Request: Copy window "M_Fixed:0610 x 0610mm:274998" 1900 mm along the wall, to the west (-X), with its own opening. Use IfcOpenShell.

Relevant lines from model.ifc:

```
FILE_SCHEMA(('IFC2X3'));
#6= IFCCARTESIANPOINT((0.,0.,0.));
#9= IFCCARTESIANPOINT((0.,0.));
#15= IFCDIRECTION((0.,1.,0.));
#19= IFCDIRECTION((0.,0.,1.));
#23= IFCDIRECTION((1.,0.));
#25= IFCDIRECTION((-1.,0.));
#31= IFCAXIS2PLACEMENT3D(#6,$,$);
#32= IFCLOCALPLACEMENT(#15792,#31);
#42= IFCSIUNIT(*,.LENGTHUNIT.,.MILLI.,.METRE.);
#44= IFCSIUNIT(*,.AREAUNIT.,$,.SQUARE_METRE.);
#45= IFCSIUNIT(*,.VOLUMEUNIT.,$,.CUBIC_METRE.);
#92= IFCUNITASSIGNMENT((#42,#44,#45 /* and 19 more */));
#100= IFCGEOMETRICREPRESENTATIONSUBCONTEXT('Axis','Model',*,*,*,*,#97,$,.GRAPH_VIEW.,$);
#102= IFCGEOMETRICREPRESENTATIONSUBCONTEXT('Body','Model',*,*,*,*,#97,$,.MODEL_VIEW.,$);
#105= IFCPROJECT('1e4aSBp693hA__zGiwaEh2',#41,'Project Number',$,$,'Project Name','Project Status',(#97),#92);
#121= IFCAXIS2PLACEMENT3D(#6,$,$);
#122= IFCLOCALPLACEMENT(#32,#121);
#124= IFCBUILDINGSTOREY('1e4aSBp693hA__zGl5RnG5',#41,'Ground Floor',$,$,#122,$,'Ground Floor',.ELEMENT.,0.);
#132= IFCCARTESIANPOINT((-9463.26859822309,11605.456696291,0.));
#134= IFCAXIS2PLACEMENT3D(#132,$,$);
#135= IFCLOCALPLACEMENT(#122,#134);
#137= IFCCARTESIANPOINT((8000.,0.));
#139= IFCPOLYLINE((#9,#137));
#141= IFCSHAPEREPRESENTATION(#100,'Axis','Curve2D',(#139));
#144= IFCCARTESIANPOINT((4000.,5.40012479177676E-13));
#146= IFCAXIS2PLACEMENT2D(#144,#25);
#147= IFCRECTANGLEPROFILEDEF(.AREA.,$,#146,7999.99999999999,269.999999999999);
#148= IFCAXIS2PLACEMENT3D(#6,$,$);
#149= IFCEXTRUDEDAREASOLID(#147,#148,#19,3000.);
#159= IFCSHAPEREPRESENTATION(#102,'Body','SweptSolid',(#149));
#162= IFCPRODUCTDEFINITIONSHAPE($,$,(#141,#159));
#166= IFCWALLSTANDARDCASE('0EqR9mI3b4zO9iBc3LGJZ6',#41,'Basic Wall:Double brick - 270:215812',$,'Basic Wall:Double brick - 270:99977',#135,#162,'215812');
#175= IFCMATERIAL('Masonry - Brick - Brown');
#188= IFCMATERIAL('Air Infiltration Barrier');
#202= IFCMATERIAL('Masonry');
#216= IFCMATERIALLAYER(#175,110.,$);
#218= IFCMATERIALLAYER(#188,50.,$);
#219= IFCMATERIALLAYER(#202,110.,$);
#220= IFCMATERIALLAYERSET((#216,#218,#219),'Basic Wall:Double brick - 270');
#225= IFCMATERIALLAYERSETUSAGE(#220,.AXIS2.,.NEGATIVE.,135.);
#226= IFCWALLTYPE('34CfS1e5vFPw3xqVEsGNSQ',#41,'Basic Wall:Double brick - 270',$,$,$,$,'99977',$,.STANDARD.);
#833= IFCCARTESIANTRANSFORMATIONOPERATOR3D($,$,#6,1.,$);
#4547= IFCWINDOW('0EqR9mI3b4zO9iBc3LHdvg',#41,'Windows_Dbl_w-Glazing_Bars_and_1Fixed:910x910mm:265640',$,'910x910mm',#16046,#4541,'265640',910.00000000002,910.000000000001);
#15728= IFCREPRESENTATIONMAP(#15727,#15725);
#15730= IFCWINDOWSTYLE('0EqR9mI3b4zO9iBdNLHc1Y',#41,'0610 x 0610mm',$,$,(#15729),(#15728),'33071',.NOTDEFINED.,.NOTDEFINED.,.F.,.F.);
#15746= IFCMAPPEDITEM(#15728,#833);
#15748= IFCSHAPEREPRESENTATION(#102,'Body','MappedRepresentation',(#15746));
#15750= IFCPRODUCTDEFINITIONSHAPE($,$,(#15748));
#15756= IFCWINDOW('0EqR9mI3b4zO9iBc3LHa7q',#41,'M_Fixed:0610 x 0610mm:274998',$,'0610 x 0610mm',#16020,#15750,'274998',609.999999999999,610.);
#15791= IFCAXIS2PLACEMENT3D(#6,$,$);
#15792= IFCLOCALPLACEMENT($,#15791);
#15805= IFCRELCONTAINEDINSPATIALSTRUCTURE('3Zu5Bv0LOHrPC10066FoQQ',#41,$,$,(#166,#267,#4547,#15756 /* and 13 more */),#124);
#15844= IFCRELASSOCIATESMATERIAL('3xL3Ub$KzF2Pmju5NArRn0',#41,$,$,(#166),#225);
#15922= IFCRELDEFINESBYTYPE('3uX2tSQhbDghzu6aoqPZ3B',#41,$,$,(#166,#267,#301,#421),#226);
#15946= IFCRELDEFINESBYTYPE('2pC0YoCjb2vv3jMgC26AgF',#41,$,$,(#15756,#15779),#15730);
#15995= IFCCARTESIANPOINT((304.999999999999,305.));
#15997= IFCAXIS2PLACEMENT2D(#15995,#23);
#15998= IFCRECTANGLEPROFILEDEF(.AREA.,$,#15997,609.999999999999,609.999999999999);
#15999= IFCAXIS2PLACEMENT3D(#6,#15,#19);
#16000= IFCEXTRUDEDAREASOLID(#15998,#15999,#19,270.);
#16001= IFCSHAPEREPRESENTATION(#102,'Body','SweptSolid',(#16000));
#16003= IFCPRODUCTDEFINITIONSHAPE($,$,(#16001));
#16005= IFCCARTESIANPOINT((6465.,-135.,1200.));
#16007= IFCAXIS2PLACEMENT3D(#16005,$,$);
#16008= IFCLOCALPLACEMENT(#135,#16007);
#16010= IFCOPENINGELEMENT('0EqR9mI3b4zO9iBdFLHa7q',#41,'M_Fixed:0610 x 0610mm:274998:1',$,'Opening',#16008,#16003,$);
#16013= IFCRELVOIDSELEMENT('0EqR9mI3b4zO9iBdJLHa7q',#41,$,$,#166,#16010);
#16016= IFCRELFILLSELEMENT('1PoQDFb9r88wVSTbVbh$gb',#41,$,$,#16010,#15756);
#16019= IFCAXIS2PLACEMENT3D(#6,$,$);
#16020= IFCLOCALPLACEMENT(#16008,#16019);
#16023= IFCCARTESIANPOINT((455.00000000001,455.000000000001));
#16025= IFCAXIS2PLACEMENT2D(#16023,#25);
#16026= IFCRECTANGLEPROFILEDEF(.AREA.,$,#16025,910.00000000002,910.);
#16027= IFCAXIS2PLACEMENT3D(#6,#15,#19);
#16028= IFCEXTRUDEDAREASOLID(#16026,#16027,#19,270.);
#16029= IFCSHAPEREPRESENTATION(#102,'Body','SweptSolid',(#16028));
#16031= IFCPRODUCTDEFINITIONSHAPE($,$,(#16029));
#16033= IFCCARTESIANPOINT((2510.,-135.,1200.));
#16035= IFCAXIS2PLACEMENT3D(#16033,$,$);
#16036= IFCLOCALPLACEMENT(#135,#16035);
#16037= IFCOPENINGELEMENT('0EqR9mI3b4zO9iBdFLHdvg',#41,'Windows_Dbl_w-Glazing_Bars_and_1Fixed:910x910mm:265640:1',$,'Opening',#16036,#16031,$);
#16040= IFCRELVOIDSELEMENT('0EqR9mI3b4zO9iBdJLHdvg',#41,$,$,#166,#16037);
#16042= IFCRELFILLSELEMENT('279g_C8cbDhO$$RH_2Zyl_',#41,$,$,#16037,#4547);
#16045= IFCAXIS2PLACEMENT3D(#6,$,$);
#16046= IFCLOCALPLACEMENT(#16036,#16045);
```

```python
import ifcopenshell
import ifcopenshell.api.feature
import ifcopenshell.api.geometry
import ifcopenshell.api.root
import ifcopenshell.geom
import ifcopenshell.util.element
import ifcopenshell.util.placement
import ifcopenshell.util.shape
import ifcopenshell.util.unit

model = ifcopenshell.open("model.ifc")
unit_scale = ifcopenshell.util.unit.calculate_unit_scale(model)
settings = ifcopenshell.geom.settings()


def volume(element):
    """Net volume in cubic metres, openings subtracted."""
    shape = ifcopenshell.geom.create_shape(settings, element)
    return ifcopenshell.util.shape.get_volume(shape.geometry)


def reuse_history(source, copy):
    """copy_class also copies each property set's owner history, people and application; keep the originals."""
    for rel in copy.IsDefinedBy:
        if rel.is_a("IfcRelDefinesByProperties") and (history := rel.RelatingPropertyDefinition.OwnerHistory):
            rel.RelatingPropertyDefinition.OwnerHistory = source.OwnerHistory
            ifcopenshell.util.element.remove_deep2(model, history)


window = model.by_guid("0EqR9mI3b4zO9iBc3LHa7q")
opening = window.FillsVoids[0].RelatingOpeningElement
wall = opening.VoidsElements[0].RelatingBuildingElement
before = volume(wall)
shift = ifcopenshell.util.placement.get_local_placement(wall.ObjectPlacement)[:3, 0] * -1.9 / unit_scale

# copy_class copies the void relationship, type, container and properties, but no geometry.
new_opening = ifcopenshell.api.root.copy_class(model, product=opening)
new_opening.Representation = ifcopenshell.util.element.copy_deep(
    model, opening.Representation, exclude=["IfcGeometricRepresentationContext", "IfcRepresentationMap"]
)
new_opening.Name = "M_Fixed:0610 x 0610mm"
new_window = ifcopenshell.api.root.copy_class(model, product=window)
new_window.Representation = ifcopenshell.util.element.copy_deep(
    model, window.Representation, exclude=["IfcGeometricRepresentationContext", "IfcRepresentationMap"]
)
new_window.Name = "M_Fixed:0610 x 0610mm"
new_window.Tag = None
reuse_history(window, new_window)
fills = ifcopenshell.api.feature.add_filling(model, opening=new_opening, element=new_window)
fills.OwnerHistory = new_window.OwnerHistory  # required in IFC2X3

for old, new in ((opening, new_opening), (window, new_window)):
    matrix = ifcopenshell.util.placement.get_local_placement(old.ObjectPlacement)
    matrix[:3, 3] += shift
    ifcopenshell.api.geometry.edit_object_placement(model, product=new, matrix=matrix, is_si=False)

after = volume(wall)

print(f"wall volume {before:.3f} -> {after:.3f} m3")

model.write("model_v2.ifc")
```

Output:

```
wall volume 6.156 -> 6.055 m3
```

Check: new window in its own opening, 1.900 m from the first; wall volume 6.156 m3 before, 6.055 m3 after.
